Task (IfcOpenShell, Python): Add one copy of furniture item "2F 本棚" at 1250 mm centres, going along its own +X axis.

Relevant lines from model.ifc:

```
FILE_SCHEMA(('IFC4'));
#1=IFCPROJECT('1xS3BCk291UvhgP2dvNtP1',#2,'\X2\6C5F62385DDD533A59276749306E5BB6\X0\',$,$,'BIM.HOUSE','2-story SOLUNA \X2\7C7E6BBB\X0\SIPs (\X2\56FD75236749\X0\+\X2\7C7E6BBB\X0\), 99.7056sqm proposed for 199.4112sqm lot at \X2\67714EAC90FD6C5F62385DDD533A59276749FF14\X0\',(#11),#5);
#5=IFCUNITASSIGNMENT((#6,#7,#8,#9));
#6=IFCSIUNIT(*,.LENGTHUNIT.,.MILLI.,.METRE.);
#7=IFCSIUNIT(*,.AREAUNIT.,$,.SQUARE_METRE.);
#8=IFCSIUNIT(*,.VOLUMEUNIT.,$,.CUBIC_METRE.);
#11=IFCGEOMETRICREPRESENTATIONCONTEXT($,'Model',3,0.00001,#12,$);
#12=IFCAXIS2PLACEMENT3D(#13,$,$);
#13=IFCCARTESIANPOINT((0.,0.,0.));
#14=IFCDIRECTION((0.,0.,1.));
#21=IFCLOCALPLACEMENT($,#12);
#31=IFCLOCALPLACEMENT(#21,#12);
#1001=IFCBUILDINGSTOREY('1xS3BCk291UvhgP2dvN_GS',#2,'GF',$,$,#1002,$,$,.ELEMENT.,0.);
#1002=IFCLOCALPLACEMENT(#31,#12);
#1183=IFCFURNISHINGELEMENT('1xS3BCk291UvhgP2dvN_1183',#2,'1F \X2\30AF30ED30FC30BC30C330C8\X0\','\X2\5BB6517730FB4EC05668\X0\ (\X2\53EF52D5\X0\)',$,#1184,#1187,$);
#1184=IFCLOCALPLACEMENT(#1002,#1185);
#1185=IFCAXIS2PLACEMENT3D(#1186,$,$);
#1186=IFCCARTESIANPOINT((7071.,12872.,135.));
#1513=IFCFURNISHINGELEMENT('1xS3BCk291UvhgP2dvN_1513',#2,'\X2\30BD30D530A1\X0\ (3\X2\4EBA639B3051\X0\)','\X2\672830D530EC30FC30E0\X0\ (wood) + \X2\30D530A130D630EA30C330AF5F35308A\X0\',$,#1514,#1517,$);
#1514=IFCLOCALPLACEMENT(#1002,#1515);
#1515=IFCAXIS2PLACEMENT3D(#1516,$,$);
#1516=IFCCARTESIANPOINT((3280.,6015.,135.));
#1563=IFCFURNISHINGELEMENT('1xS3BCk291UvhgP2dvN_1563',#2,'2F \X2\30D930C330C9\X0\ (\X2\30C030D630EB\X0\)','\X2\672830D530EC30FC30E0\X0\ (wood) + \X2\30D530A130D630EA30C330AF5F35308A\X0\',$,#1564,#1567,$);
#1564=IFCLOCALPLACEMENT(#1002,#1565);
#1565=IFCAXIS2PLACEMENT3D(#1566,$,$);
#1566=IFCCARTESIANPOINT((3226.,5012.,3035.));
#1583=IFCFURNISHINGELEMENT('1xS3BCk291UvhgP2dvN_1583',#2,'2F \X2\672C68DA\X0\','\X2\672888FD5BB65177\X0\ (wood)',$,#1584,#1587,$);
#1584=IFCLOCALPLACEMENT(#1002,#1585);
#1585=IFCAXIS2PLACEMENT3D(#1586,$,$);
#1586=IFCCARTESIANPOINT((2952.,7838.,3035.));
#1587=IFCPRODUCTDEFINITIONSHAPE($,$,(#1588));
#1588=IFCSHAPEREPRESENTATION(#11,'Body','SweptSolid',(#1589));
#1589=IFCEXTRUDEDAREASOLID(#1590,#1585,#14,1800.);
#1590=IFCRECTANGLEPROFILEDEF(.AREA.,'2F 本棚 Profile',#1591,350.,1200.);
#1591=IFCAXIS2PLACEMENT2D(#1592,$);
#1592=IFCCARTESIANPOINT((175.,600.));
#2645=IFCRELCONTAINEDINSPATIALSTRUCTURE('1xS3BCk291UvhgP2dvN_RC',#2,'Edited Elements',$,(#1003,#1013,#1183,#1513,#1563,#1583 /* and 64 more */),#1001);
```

```python
import ifcopenshell
import ifcopenshell.api.geometry
import ifcopenshell.api.root
import ifcopenshell.util.element
import ifcopenshell.util.placement
import ifcopenshell.util.unit

model = ifcopenshell.open("model.ifc")
unit_scale = ifcopenshell.util.unit.calculate_unit_scale(model)


def reuse_history(source, copy):
    """copy_class also copies each property set's owner history, people and application; keep the originals."""
    for rel in copy.IsDefinedBy:
        if rel.is_a("IfcRelDefinesByProperties") and (history := rel.RelatingPropertyDefinition.OwnerHistory):
            rel.RelatingPropertyDefinition.OwnerHistory = source.OwnerHistory
            ifcopenshell.util.element.remove_deep2(model, history)


source = model.by_guid("1xS3BCk291UvhgP2dvN_1583")
base = ifcopenshell.util.placement.get_local_placement(source.ObjectPlacement)
step = base[:3, 0] * 1.25 / unit_scale

for i in range(1, 2):
    copy = ifcopenshell.api.root.copy_class(model, product=source)
    copy.Representation = ifcopenshell.util.element.copy_deep(
        model, source.Representation, exclude=["IfcGeometricRepresentationContext", "IfcRepresentationMap"]
    )
    reuse_history(source, copy)
    matrix = base.copy()
    matrix[:3, 3] += i * step
    print("added at", matrix[:3, 3].round(3) + 0.0)
    ifcopenshell.api.geometry.edit_object_placement(model, product=copy, matrix=matrix, is_si=False)

model.write("model-out.ifc")
```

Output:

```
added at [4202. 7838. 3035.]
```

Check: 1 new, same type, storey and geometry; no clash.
